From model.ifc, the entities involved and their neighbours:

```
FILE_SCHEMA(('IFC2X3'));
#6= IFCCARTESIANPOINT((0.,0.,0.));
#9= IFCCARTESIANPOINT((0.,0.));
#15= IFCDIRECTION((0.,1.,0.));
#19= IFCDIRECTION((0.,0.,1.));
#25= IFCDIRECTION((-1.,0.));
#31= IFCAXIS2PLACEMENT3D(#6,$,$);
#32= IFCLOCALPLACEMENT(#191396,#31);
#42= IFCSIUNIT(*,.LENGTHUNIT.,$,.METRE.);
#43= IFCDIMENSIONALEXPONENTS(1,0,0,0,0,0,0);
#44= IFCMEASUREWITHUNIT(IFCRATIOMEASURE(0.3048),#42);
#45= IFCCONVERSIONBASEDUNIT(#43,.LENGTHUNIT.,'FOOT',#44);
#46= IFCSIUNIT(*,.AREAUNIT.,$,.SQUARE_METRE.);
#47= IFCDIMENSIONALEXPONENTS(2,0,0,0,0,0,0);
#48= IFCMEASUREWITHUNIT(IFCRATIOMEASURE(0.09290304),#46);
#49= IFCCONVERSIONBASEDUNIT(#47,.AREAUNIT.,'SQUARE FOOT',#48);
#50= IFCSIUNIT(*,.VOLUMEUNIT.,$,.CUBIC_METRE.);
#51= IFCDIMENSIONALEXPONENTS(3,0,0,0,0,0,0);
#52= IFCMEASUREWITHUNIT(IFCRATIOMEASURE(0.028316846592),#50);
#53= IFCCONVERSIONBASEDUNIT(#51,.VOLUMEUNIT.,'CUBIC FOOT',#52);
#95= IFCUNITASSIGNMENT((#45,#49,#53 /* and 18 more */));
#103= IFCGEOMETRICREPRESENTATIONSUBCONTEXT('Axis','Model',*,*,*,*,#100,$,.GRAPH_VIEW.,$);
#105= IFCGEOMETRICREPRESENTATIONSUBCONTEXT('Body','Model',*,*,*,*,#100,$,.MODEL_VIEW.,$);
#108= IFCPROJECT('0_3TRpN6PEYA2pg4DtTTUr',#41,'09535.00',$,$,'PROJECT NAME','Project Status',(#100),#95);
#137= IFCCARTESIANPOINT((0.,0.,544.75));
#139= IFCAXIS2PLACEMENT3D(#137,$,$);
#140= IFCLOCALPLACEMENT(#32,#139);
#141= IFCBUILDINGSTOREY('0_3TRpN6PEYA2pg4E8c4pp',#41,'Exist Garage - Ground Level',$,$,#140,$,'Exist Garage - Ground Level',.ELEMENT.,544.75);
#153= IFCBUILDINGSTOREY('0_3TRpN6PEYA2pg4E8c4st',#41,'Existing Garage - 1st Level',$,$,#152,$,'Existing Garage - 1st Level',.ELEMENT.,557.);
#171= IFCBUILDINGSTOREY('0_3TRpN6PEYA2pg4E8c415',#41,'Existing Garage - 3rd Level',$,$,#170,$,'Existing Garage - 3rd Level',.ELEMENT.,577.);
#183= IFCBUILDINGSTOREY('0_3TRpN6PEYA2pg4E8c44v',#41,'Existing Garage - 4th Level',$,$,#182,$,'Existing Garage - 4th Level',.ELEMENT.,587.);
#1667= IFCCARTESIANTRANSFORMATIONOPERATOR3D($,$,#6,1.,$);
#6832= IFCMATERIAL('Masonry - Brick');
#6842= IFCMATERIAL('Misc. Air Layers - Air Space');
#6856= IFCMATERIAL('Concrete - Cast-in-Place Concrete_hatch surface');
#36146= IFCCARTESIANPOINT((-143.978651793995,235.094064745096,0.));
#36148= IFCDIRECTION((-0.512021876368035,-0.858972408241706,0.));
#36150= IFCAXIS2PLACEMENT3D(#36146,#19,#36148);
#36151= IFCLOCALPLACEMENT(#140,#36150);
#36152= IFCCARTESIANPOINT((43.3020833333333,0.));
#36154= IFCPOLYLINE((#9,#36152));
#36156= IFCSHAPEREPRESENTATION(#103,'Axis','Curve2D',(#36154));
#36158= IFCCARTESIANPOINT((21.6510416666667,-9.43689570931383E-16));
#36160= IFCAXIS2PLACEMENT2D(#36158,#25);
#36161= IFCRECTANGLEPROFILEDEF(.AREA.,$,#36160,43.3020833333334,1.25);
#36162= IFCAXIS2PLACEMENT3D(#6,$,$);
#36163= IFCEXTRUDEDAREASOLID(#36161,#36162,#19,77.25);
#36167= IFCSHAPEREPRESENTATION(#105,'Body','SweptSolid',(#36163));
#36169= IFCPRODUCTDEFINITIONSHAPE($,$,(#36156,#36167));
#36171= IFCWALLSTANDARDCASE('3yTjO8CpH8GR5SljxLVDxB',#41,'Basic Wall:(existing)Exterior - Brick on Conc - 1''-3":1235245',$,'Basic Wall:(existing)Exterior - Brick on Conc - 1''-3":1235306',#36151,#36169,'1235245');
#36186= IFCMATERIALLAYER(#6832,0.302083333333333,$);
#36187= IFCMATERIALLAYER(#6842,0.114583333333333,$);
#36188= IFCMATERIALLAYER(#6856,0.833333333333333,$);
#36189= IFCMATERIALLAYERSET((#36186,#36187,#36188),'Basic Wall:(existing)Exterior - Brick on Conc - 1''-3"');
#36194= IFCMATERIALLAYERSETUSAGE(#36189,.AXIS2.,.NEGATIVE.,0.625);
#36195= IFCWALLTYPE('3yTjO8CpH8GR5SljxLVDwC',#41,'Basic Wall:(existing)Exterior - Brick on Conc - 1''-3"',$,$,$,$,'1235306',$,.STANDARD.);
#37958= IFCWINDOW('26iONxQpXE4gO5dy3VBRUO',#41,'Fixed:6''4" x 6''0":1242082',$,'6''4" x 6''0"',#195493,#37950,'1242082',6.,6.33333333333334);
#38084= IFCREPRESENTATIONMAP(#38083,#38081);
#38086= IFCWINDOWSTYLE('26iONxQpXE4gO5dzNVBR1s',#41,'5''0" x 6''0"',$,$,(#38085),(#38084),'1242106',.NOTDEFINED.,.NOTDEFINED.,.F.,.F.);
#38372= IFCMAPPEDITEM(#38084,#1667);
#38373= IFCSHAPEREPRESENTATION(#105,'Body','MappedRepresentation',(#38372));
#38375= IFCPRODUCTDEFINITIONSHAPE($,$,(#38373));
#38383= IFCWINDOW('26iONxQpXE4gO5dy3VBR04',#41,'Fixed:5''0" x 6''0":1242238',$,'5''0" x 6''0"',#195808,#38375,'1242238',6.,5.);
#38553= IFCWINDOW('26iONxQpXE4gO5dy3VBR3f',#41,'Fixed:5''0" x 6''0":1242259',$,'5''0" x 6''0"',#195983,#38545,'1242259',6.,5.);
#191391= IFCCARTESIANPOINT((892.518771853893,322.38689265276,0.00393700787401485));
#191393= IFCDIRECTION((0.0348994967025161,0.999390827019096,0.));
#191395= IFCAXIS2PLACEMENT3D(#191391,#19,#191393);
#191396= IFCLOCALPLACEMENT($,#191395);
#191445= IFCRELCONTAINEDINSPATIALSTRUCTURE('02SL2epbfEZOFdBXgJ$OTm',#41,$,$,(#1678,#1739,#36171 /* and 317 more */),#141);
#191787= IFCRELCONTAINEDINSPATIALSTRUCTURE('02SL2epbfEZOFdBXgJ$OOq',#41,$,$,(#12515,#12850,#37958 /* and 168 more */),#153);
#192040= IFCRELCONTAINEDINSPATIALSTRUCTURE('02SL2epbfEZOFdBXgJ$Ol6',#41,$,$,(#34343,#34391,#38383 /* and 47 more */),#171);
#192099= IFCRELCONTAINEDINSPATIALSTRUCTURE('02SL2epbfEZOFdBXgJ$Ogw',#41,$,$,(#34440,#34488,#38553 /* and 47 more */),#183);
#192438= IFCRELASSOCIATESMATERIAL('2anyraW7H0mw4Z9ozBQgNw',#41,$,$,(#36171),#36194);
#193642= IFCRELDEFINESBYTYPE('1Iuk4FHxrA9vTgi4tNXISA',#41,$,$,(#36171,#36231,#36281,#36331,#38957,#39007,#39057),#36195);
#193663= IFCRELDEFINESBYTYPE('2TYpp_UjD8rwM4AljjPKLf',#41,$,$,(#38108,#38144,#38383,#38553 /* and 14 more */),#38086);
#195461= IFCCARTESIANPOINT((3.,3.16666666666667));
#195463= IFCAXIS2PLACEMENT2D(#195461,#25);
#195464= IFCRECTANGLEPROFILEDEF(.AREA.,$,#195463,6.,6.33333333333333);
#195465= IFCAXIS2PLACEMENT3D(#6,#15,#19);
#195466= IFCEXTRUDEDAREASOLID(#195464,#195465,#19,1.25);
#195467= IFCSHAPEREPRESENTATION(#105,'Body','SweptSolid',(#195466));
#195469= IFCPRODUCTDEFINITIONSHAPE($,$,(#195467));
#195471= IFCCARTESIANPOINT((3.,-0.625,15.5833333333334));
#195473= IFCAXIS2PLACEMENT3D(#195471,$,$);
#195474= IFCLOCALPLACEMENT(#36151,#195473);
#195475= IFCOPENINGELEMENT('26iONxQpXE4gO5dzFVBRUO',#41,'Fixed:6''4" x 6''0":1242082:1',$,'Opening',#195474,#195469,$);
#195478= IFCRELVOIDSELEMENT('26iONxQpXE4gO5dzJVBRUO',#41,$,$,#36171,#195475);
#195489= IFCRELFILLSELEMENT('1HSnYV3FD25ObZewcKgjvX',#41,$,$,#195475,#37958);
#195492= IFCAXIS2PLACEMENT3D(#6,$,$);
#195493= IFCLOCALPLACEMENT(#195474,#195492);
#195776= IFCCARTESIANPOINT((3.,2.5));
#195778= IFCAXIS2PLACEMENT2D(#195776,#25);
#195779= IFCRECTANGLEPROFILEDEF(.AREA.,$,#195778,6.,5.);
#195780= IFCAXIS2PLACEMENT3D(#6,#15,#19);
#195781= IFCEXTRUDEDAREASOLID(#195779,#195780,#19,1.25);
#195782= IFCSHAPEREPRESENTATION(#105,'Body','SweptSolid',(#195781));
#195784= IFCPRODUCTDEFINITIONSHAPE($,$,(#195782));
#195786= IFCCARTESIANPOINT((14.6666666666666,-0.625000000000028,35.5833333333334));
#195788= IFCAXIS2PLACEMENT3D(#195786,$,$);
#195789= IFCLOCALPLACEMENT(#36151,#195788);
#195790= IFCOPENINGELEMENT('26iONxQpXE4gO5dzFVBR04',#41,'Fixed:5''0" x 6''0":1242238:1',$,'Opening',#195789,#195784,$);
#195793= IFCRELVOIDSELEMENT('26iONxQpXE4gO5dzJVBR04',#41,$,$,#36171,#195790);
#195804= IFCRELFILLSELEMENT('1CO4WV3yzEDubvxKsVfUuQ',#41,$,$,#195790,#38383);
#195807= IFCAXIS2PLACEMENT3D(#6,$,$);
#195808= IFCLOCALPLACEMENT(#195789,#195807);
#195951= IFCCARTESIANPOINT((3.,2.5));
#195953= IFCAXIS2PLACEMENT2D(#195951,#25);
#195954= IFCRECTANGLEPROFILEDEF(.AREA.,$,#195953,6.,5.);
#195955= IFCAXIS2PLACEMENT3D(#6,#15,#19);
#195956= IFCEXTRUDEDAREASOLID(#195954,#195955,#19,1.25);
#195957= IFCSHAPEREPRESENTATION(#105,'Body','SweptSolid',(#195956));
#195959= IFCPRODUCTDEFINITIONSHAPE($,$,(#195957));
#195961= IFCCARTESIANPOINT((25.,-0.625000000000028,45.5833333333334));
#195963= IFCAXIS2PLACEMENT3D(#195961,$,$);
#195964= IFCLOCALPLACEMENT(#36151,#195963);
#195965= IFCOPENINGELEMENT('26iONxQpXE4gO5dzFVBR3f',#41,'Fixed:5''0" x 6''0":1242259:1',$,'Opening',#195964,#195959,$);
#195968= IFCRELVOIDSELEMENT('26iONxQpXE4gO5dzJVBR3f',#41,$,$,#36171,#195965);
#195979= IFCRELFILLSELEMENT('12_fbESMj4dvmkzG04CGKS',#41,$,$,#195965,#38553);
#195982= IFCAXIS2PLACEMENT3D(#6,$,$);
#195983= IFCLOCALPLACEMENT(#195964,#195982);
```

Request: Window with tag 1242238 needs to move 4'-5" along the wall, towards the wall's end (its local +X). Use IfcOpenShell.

```python
import ifcopenshell
import ifcopenshell.api.geometry
import ifcopenshell.util.placement
import ifcopenshell.util.unit

model = ifcopenshell.open("model.ifc")
unit_scale = ifcopenshell.util.unit.calculate_unit_scale(model)

window = model.by_id(38383)
opening = window.FillsVoids[0].RelatingOpeningElement
wall = opening.VoidsElements[0].RelatingBuildingElement

wall_matrix = ifcopenshell.util.placement.get_local_placement(wall.ObjectPlacement)
shift = wall_matrix[:3, 0] * 53 * 0.0254 / unit_scale
before = ifcopenshell.util.placement.get_local_placement(window.ObjectPlacement)[:3, 3].copy()

# The window is placed relative to its opening, so it follows when the opening moves.
matrix = ifcopenshell.util.placement.get_local_placement(opening.ObjectPlacement)
matrix[:3, 3] += shift
ifcopenshell.api.geometry.edit_object_placement(
    model, product=opening, matrix=matrix, is_si=False, should_transform_children=True
)

after = ifcopenshell.util.placement.get_local_placement(window.ObjectPlacement)[:3, 3]
print("window moved by", (after - before).round(3) + 0.0)

model.write("model_edited.ifc")
```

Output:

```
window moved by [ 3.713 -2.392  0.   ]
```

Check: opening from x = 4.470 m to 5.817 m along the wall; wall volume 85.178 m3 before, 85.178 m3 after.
